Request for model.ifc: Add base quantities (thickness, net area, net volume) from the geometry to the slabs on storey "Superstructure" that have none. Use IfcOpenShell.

First a look at what the model holds.

```python
import ifcopenshell
import ifcopenshell.util.element
import ifcopenshell.util.unit

model = ifcopenshell.open("model.ifc")
print(model.schema)
for unit_type in ("LENGTHUNIT", "AREAUNIT", "VOLUMEUNIT"):
    print(unit_type, ifcopenshell.util.unit.calculate_unit_scale(model, unit_type))
storey = next(s for s in model.by_type("IfcBuildingStorey") if s.Name == "Superstructure")
slabs = [e for e in ifcopenshell.util.element.get_decomposition(storey) if e.is_a("IfcSlab")]
for e in sorted(slabs, key=lambda e: e.id()):
    print(e.id(), e.is_a(), e.Name, list(ifcopenshell.util.element.get_psets(e, qtos_only=True)), sep=" | ")
```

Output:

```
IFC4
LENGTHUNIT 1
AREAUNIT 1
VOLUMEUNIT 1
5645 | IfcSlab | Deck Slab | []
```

```python
import ifcopenshell
import ifcopenshell.api.pset
import ifcopenshell.geom
import ifcopenshell.util.element
import ifcopenshell.util.shape
import ifcopenshell.util.unit

model = ifcopenshell.open("model.ifc")
unit_scale = ifcopenshell.util.unit.calculate_unit_scale(model)
area_scale = ifcopenshell.util.unit.calculate_unit_scale(model, "AREAUNIT")
volume_scale = ifcopenshell.util.unit.calculate_unit_scale(model, "VOLUMEUNIT")
settings = ifcopenshell.geom.settings()

storey = next(s for s in model.by_type("IfcBuildingStorey") if s.Name == "Superstructure")
slabs = [e for e in ifcopenshell.util.element.get_decomposition(storey) if e.is_a("IfcSlab")]

for e in sorted(slabs, key=lambda e: e.id()):
    if ifcopenshell.util.element.get_psets(e, qtos_only=True, should_inherit=False):
        continue
    # Geometry comes back in metres, in the element's own axes.
    shape = ifcopenshell.geom.create_shape(settings, e)
    values = {
        "Width": ifcopenshell.util.shape.get_z(shape.geometry) / unit_scale,
        "NetArea": ifcopenshell.util.shape.get_footprint_area(shape.geometry) / area_scale,
        "NetVolume": ifcopenshell.util.shape.get_volume(shape.geometry) / volume_scale,
    }
    qto = ifcopenshell.api.pset.add_qto(model, product=e, name="Qto_SlabBaseQuantities")
    ifcopenshell.api.pset.edit_qto(model, qto=qto, properties=values)
    print(e.id(), {k: round(v, 3) for k, v in values.items()})

model.write("model_rev.ifc")
```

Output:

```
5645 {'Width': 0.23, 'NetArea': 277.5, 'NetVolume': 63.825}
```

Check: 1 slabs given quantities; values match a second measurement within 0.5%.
